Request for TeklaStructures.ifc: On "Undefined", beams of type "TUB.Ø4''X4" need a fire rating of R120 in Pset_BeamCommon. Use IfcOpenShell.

First a look at what the model holds.

```python
import ifcopenshell
import ifcopenshell.util.element

model = ifcopenshell.open("TeklaStructures.ifc")
print(model.schema)
storey = next(s for s in model.by_type("IfcBuildingStorey") if s.Name == "Undefined")
beams = [e for e in ifcopenshell.util.element.get_decomposition(storey) if e.is_a("IfcBeam")]
seen = {}
for e in beams:
    element_type = ifcopenshell.util.element.get_type(e)
    key = (element_type.Name if element_type != e and element_type else None, ifcopenshell.util.element.get_pset(e, "Pset_BeamCommon", "FireRating"))
    seen[key] = seen.get(key, 0) + 1
for (name, value), count in sorted(seen.items(), key=str):
    print(count, "x", name, "|", value)
```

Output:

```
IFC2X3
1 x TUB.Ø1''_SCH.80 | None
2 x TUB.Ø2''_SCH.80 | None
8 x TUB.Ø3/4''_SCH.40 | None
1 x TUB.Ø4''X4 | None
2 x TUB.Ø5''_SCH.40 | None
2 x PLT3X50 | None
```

```python
import ifcopenshell
import ifcopenshell.api.pset
import ifcopenshell.util.element

model = ifcopenshell.open("TeklaStructures.ifc")

storey = next(s for s in model.by_type("IfcBuildingStorey") if s.Name == "Undefined")
beams = [e for e in ifcopenshell.util.element.get_decomposition(storey) if e.is_a("IfcBeam")]

count = 0
for e in beams:
    element_type = ifcopenshell.util.element.get_type(e)
    if element_type in (None, e) or element_type.Name != "TUB.Ø4''X4":
        continue
    # add_pset returns the element's existing set when there is one.
    pset = ifcopenshell.api.pset.add_pset(model, product=e, name="Pset_BeamCommon")
    ifcopenshell.api.pset.edit_pset(model, pset=pset, properties={"FireRating": "R120"})
    count += 1

print(count, "beams updated")

model.write("TeklaStructures-out.ifc")
```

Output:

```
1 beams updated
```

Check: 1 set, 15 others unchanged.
